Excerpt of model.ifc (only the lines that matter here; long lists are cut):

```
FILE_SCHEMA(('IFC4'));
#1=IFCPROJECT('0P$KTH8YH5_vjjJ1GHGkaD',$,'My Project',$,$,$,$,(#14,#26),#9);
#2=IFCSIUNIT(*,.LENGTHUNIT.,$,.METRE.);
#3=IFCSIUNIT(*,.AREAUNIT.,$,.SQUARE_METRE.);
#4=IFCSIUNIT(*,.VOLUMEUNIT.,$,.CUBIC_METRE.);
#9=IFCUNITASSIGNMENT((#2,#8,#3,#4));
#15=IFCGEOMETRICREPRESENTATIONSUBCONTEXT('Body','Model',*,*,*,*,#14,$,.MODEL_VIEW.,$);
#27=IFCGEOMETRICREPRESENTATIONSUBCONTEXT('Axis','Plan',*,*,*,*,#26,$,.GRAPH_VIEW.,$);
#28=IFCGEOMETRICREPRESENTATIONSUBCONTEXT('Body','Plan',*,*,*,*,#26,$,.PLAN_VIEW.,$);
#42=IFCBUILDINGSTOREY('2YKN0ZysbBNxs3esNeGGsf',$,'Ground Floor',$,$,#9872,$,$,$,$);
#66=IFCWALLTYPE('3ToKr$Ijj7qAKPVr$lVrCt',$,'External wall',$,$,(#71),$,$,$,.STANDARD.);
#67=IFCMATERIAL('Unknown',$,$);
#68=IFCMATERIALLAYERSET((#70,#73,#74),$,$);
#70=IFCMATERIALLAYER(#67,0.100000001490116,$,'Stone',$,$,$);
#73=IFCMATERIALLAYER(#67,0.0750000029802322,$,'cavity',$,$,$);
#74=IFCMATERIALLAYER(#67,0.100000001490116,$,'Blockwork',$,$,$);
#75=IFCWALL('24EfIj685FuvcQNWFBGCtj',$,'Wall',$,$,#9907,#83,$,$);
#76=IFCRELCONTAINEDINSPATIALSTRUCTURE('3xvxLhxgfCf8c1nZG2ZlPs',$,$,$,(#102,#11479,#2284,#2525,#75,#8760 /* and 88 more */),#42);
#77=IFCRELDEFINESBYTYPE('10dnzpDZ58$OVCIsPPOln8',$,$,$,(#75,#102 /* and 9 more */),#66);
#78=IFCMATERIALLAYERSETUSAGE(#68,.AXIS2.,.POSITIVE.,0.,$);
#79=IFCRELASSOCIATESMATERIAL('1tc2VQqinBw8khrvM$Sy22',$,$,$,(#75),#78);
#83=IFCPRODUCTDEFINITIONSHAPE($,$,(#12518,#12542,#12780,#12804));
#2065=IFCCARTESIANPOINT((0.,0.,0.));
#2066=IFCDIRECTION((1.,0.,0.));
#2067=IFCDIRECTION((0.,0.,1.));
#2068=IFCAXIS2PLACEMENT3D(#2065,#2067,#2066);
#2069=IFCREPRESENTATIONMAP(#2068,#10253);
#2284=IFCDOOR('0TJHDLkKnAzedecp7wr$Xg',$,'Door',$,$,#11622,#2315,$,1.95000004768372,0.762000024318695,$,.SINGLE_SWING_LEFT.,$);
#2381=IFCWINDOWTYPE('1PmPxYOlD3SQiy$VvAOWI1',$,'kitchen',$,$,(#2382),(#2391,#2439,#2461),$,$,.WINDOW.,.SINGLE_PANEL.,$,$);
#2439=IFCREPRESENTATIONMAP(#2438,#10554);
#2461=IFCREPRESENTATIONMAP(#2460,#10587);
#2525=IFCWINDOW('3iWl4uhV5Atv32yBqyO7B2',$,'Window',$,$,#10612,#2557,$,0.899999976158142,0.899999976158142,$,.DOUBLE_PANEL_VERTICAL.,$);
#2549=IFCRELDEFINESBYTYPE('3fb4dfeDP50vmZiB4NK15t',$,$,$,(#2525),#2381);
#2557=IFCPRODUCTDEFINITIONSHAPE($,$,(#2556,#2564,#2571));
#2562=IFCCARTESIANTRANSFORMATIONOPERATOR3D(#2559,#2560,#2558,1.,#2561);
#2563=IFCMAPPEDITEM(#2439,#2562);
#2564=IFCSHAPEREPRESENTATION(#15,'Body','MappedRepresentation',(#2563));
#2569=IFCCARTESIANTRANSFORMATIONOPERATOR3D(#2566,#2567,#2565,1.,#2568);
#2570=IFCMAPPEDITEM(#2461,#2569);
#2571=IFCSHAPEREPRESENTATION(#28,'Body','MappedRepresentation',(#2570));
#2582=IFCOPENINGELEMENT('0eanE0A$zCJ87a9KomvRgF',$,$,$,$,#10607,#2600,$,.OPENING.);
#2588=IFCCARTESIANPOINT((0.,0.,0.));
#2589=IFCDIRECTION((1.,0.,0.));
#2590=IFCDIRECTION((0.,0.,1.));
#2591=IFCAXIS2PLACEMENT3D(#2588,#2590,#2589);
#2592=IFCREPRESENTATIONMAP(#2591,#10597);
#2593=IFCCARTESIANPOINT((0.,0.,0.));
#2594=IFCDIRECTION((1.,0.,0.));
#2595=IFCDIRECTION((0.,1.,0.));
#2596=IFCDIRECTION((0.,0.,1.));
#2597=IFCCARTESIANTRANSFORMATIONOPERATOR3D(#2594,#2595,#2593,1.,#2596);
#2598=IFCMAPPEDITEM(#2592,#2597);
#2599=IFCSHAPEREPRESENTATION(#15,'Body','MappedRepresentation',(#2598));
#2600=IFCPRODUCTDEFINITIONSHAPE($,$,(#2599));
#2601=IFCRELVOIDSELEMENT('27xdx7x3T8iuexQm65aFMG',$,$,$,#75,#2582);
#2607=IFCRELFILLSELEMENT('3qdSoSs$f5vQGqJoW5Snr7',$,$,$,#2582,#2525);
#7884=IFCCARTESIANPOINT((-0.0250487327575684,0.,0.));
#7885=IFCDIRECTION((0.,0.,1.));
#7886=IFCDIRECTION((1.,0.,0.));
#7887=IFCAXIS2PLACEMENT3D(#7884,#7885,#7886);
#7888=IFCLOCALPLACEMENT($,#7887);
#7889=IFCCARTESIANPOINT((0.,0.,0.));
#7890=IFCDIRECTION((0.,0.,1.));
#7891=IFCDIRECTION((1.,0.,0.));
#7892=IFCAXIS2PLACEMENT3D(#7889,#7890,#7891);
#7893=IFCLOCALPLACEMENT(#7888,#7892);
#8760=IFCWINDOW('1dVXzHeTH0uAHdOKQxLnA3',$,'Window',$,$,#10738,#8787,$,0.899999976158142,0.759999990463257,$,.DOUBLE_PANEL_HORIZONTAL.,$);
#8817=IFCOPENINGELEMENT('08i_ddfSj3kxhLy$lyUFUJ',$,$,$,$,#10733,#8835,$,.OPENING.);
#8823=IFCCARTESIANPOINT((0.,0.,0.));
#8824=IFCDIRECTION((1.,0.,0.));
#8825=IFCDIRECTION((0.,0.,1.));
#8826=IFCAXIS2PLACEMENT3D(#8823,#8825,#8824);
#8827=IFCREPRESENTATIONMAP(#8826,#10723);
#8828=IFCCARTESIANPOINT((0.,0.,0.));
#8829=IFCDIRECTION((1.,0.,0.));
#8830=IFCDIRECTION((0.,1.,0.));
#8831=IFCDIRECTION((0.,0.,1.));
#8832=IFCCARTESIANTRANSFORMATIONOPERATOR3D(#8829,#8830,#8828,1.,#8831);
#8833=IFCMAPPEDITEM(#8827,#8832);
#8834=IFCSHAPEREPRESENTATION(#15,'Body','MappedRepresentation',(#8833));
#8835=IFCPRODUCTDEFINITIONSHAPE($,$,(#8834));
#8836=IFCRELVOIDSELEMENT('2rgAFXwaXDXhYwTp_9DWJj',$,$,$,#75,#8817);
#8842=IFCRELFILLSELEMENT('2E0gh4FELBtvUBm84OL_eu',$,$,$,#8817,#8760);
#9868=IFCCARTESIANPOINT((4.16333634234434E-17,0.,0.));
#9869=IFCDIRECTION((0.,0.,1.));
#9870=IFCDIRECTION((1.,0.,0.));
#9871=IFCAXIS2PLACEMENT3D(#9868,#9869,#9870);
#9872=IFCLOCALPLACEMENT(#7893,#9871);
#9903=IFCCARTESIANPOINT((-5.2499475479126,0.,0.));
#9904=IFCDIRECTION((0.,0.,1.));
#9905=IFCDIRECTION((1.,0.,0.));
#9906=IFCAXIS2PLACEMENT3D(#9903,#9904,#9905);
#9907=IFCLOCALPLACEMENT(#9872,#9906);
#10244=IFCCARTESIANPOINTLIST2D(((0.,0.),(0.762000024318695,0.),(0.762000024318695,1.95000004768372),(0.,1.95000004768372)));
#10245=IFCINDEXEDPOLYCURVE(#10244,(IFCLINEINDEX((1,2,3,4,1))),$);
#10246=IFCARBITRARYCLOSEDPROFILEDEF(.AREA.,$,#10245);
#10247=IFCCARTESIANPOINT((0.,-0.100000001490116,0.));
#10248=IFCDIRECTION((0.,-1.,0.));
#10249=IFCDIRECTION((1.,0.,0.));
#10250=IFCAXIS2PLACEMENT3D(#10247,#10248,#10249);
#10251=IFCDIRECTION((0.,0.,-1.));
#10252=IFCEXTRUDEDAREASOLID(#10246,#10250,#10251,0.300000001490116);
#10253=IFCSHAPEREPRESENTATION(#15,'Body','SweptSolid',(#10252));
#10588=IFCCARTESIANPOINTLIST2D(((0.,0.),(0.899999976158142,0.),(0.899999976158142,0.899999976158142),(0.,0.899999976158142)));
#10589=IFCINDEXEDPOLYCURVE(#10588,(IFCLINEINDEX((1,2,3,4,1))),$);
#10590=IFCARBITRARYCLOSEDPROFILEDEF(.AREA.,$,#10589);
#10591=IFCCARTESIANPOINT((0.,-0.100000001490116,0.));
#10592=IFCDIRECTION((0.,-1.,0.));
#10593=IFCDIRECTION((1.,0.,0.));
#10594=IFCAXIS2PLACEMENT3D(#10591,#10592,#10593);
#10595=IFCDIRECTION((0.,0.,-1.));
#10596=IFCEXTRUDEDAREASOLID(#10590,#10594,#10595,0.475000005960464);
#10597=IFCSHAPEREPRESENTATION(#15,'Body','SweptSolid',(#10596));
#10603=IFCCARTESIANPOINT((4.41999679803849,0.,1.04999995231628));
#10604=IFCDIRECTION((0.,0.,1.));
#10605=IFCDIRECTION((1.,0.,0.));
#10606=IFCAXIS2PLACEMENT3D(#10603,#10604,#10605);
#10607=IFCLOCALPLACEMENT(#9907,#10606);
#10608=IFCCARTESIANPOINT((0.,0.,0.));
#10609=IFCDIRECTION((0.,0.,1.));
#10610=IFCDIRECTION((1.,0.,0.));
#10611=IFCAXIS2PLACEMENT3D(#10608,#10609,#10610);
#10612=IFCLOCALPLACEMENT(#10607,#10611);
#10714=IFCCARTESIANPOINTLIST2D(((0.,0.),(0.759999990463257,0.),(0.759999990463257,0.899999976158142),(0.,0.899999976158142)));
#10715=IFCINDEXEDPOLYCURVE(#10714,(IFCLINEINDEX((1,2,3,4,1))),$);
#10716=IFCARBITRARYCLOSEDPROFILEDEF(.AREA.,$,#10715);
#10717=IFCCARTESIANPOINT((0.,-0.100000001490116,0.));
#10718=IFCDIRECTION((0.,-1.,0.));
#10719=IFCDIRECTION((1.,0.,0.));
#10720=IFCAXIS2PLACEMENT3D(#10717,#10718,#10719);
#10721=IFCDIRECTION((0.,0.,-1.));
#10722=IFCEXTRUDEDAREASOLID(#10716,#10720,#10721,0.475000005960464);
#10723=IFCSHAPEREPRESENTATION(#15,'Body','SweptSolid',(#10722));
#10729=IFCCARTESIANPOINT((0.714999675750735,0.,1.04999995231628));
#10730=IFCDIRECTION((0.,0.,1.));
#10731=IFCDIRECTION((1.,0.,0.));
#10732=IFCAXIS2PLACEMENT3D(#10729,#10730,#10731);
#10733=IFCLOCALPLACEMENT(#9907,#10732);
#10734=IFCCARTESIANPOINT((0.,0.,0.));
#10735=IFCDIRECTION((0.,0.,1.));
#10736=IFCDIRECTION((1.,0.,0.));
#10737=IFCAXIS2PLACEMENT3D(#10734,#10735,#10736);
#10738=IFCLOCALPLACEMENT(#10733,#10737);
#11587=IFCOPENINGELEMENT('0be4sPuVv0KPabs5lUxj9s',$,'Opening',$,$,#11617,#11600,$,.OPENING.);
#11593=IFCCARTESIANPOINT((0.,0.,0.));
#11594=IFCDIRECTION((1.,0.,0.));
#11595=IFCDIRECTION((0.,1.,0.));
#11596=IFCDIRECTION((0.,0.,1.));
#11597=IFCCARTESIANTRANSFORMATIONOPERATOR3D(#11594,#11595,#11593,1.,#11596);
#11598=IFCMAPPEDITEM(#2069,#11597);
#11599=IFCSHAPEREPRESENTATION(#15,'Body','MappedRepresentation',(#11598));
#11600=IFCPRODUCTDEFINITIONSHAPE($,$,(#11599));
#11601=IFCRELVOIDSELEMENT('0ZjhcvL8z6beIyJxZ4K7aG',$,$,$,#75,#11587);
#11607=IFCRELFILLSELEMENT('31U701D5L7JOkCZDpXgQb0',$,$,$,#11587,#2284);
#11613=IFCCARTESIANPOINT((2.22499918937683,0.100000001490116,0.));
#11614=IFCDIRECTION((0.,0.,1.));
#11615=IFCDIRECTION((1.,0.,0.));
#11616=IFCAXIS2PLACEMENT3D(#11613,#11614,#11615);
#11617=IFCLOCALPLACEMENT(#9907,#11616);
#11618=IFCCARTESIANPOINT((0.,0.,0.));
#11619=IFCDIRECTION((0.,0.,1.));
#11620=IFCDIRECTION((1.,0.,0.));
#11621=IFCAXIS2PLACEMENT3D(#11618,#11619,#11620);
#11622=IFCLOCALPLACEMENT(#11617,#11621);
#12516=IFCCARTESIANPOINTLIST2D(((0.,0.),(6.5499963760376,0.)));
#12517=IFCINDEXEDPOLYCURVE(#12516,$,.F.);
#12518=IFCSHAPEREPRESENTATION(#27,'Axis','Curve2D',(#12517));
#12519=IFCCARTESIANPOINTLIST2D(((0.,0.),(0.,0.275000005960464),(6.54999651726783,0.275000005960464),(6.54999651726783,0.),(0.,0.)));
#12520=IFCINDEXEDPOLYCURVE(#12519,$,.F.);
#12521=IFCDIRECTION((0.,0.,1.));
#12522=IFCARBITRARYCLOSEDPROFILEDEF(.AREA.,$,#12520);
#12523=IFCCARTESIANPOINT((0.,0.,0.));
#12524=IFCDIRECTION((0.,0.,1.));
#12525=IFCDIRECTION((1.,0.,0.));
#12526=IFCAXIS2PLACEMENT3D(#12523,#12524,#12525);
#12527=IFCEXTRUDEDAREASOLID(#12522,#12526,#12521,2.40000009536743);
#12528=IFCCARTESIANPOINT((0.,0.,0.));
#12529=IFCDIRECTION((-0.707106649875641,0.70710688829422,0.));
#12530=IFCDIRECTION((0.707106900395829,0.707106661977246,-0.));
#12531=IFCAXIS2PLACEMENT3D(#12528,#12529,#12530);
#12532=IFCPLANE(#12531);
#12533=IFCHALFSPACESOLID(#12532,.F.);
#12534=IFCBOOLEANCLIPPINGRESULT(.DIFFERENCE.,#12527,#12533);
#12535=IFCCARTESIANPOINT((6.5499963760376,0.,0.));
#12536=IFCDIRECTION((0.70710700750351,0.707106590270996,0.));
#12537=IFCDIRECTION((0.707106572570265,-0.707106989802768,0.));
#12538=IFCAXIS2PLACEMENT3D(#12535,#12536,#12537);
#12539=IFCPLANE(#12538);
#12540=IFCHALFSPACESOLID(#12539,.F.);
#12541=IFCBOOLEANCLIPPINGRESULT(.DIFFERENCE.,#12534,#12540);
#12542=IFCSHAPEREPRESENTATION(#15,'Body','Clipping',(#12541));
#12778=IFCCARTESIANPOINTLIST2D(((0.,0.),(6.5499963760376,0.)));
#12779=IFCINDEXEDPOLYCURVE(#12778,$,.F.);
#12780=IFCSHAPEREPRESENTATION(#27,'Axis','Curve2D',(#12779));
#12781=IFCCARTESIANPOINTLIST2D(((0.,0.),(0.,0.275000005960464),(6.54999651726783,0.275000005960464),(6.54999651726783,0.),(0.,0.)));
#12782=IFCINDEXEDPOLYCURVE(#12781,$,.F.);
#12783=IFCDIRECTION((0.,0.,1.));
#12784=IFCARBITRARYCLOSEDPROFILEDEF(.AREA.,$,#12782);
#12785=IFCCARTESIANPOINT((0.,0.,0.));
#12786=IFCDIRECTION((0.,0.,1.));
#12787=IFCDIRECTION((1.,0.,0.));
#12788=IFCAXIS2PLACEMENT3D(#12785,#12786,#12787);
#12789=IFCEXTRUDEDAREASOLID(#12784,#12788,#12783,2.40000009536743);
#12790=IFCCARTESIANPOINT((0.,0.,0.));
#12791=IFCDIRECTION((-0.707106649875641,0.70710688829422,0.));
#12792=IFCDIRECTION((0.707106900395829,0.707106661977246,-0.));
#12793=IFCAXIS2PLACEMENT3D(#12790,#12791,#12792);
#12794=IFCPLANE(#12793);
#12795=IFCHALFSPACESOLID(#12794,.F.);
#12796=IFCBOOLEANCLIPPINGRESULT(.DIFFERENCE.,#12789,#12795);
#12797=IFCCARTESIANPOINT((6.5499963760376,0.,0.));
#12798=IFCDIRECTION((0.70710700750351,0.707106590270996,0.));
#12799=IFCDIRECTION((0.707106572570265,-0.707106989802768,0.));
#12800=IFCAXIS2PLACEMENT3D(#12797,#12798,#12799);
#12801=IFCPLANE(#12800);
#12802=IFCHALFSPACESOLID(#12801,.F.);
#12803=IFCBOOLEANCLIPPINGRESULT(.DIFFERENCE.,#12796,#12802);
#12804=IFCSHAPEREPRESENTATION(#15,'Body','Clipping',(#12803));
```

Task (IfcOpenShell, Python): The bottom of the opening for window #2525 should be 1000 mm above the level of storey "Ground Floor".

```python
import numpy as np
import ifcopenshell
import ifcopenshell.api.geometry
import ifcopenshell.geom
import ifcopenshell.util.element
import ifcopenshell.util.placement
import ifcopenshell.util.shape
import ifcopenshell.util.unit

model = ifcopenshell.open("model.ifc")
unit_scale = ifcopenshell.util.unit.calculate_unit_scale(model)

window = model.by_guid("3iWl4uhV5Atv32yBqyO7B2")
opening = window.FillsVoids[0].RelatingOpeningElement
storey = ifcopenshell.util.element.get_container(window, ifc_class="IfcBuildingStorey")
level = ifcopenshell.util.placement.get_local_placement(storey.ObjectPlacement)[2, 3]

# The opening's origin need not be at the sill, so measure its lowest point.
shape = ifcopenshell.geom.create_shape(ifcopenshell.geom.settings(), opening)
bottom = ifcopenshell.util.shape.get_shape_bottom_elevation(shape, shape.geometry) / unit_scale
dz = level + 1 / unit_scale - bottom

shift = np.array([0.0, 0.0, dz])
# The window is placed relative to its opening, so it follows when the opening moves.
matrix = ifcopenshell.util.placement.get_local_placement(opening.ObjectPlacement)
matrix[:3, 3] += shift
ifcopenshell.api.geometry.edit_object_placement(
    model, product=opening, matrix=matrix, is_si=False, should_transform_children=True
)

print(f"moved by {dz * unit_scale:+.3f} m")

model.write("model-out.ifc")
```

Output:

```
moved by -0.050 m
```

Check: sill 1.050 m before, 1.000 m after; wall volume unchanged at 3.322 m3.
